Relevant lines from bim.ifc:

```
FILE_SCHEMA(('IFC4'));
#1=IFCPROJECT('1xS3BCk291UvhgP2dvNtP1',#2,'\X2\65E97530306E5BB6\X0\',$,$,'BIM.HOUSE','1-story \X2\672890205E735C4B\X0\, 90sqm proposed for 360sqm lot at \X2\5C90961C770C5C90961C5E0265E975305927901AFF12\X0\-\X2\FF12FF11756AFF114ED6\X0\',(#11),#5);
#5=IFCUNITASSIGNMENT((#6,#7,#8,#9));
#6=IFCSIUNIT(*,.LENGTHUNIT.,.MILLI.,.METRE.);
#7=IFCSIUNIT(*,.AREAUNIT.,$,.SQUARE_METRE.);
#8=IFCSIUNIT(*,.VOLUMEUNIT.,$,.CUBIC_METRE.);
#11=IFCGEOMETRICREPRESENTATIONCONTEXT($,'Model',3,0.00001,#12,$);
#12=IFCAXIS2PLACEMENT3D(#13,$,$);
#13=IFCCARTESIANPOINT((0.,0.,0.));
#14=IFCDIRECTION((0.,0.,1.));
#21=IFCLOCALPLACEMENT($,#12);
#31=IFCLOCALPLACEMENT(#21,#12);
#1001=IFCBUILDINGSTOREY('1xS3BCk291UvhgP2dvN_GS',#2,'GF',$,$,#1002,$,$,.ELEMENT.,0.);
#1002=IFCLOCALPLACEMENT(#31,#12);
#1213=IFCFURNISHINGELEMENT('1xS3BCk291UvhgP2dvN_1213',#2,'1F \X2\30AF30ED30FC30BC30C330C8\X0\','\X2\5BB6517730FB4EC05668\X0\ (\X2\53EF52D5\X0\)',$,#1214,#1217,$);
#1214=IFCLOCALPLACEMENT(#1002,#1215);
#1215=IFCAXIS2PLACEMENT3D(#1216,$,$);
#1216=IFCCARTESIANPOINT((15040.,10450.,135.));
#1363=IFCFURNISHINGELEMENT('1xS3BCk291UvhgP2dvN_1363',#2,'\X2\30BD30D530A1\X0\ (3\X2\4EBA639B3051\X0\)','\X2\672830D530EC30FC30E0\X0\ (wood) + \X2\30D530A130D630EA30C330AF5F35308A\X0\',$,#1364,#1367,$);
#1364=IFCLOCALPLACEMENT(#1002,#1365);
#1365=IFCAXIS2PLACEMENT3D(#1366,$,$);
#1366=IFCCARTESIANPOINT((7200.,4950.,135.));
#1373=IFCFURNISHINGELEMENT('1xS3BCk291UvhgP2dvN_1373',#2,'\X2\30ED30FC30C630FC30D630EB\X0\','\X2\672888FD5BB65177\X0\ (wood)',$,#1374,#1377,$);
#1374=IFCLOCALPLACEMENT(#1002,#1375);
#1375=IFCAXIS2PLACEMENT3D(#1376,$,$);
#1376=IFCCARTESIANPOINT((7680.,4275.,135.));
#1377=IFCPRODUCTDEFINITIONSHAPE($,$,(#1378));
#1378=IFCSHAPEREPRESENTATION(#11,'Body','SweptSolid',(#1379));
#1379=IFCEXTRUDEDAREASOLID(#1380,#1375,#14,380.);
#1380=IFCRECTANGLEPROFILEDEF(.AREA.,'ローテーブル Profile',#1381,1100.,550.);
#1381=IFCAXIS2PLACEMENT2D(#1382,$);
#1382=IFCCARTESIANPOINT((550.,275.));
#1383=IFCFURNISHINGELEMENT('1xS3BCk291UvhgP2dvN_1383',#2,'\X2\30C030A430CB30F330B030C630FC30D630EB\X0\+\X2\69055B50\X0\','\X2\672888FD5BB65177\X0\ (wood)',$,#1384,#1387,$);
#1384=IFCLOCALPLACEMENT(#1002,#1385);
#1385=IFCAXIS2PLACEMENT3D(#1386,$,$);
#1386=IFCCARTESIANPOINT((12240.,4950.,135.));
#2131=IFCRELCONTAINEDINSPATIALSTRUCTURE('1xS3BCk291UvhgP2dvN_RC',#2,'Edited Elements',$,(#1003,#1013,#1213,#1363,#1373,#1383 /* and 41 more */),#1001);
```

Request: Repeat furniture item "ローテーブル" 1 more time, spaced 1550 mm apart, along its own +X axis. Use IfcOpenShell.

```python
import ifcopenshell
import ifcopenshell.api.geometry
import ifcopenshell.api.root
import ifcopenshell.util.element
import ifcopenshell.util.placement
import ifcopenshell.util.unit

model = ifcopenshell.open("bim.ifc")
unit_scale = ifcopenshell.util.unit.calculate_unit_scale(model)


def reuse_history(source, copy):
    """copy_class also copies each property set's owner history, people and application; keep the originals."""
    for rel in copy.IsDefinedBy:
        if rel.is_a("IfcRelDefinesByProperties") and (history := rel.RelatingPropertyDefinition.OwnerHistory):
            rel.RelatingPropertyDefinition.OwnerHistory = source.OwnerHistory
            ifcopenshell.util.element.remove_deep2(model, history)


source = model.by_guid("1xS3BCk291UvhgP2dvN_1373")
base = ifcopenshell.util.placement.get_local_placement(source.ObjectPlacement)
step = base[:3, 0] * 1.55 / unit_scale

for i in range(1, 2):
    copy = ifcopenshell.api.root.copy_class(model, product=source)
    copy.Representation = ifcopenshell.util.element.copy_deep(
        model, source.Representation, exclude=["IfcGeometricRepresentationContext", "IfcRepresentationMap"]
    )
    reuse_history(source, copy)
    matrix = base.copy()
    matrix[:3, 3] += i * step
    print("added at", matrix[:3, 3].round(3) + 0.0)
    ifcopenshell.api.geometry.edit_object_placement(model, product=copy, matrix=matrix, is_si=False)

model.write("bim_updated.ifc")
```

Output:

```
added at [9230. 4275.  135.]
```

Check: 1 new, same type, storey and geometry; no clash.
